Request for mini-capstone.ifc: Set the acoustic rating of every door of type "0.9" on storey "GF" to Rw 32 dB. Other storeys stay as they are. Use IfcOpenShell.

First a look at what the model holds.

```python
import ifcopenshell
import ifcopenshell.util.element

model = ifcopenshell.open("mini-capstone.ifc")
print(model.schema)
storey = next(s for s in model.by_type("IfcBuildingStorey") if s.Name == "GF")
doors = [e for e in ifcopenshell.util.element.get_decomposition(storey) if e.is_a("IfcDoor")]
seen = {}
for e in doors:
    element_type = ifcopenshell.util.element.get_type(e)
    key = (element_type.Name if element_type != e and element_type else None, ifcopenshell.util.element.get_pset(e, "Pset_DoorCommon", "AcousticRating"))
    seen[key] = seen.get(key, 0) + 1
for (name, value), count in sorted(seen.items(), key=str):
    print(count, "x", name, "|", value)
```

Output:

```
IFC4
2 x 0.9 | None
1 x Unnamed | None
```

```python
import ifcopenshell
import ifcopenshell.api.pset
import ifcopenshell.util.element

model = ifcopenshell.open("mini-capstone.ifc")

storey = next(s for s in model.by_type("IfcBuildingStorey") if s.Name == "GF")
doors = [e for e in ifcopenshell.util.element.get_decomposition(storey) if e.is_a("IfcDoor")]

count = 0
for e in doors:
    element_type = ifcopenshell.util.element.get_type(e)
    if element_type in (None, e) or element_type.Name != "0.9":
        continue
    # add_pset returns the element's existing set when there is one.
    pset = ifcopenshell.api.pset.add_pset(model, product=e, name="Pset_DoorCommon")
    ifcopenshell.api.pset.edit_pset(model, pset=pset, properties={"AcousticRating": "Rw 32 dB"})
    count += 1

print(count, "doors updated")

model.write("mini-capstone_updated.ifc")
```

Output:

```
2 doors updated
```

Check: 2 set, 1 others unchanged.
